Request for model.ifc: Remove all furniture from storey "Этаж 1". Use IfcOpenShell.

First a look at what the model holds.

```python
import ifcopenshell
import ifcopenshell.util.element

model = ifcopenshell.open("model.ifc")
print(model.schema)
storey = next(s for s in model.by_type("IfcBuildingStorey") if s.Name == "Этаж 1")
furniture = [e for e in ifcopenshell.util.element.get_decomposition(storey) if e.is_a("IfcFurnishingElement")]
seen = {}
for e in furniture:
    element_type = ifcopenshell.util.element.get_type(e)
    name = element_type.Name if element_type not in (None, e) else None
    seen[name] = seen.get(name, 0) + 1
for name, count in sorted(seen.items(), key=str):
    print(count, "x", name)
```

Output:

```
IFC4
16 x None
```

```python
import ifcopenshell
import ifcopenshell.api.root
import ifcopenshell.util.element

model = ifcopenshell.open("model.ifc")

storey = next(s for s in model.by_type("IfcBuildingStorey") if s.Name == "Этаж 1")
furniture = [e for e in ifcopenshell.util.element.get_decomposition(storey) if e.is_a("IfcFurnishingElement")]

for e in furniture:
    ifcopenshell.api.root.remove_product(model, product=e)
print(len(furniture), "removed")

model.write("model_edited.ifc")
```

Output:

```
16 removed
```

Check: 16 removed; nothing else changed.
